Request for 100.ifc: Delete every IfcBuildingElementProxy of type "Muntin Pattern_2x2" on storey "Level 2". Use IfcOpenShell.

First a look at what the model holds.

```python
import ifcopenshell
import ifcopenshell.util.element

model = ifcopenshell.open("100.ifc")
print(model.schema)
storey = next(s for s in model.by_type("IfcBuildingStorey") if s.Name == "Level 2")
proxies = [e for e in ifcopenshell.util.element.get_decomposition(storey) if e.is_a("IfcBuildingElementProxy")]
seen = {}
for e in proxies:
    element_type = ifcopenshell.util.element.get_type(e)
    name = element_type.Name if element_type not in (None, e) else None
    seen[name] = seen.get(name, 0) + 1
for name, count in sorted(seen.items(), key=str):
    print(count, "x", name)
```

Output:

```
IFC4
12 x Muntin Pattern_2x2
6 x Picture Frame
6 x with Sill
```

```python
import ifcopenshell
import ifcopenshell.api.root
import ifcopenshell.util.element

model = ifcopenshell.open("100.ifc")

storey = next(s for s in model.by_type("IfcBuildingStorey") if s.Name == "Level 2")
proxies = [e for e in ifcopenshell.util.element.get_decomposition(storey) if e.is_a("IfcBuildingElementProxy")]
targets = [e for e in proxies if (t := ifcopenshell.util.element.get_type(e)) not in (None, e) and t.Name == "Muntin Pattern_2x2"]

for e in targets:
    ifcopenshell.api.root.remove_product(model, product=e)
print(len(targets), "removed")

model.write("100_v2.ifc")
```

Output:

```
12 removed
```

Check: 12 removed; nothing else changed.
